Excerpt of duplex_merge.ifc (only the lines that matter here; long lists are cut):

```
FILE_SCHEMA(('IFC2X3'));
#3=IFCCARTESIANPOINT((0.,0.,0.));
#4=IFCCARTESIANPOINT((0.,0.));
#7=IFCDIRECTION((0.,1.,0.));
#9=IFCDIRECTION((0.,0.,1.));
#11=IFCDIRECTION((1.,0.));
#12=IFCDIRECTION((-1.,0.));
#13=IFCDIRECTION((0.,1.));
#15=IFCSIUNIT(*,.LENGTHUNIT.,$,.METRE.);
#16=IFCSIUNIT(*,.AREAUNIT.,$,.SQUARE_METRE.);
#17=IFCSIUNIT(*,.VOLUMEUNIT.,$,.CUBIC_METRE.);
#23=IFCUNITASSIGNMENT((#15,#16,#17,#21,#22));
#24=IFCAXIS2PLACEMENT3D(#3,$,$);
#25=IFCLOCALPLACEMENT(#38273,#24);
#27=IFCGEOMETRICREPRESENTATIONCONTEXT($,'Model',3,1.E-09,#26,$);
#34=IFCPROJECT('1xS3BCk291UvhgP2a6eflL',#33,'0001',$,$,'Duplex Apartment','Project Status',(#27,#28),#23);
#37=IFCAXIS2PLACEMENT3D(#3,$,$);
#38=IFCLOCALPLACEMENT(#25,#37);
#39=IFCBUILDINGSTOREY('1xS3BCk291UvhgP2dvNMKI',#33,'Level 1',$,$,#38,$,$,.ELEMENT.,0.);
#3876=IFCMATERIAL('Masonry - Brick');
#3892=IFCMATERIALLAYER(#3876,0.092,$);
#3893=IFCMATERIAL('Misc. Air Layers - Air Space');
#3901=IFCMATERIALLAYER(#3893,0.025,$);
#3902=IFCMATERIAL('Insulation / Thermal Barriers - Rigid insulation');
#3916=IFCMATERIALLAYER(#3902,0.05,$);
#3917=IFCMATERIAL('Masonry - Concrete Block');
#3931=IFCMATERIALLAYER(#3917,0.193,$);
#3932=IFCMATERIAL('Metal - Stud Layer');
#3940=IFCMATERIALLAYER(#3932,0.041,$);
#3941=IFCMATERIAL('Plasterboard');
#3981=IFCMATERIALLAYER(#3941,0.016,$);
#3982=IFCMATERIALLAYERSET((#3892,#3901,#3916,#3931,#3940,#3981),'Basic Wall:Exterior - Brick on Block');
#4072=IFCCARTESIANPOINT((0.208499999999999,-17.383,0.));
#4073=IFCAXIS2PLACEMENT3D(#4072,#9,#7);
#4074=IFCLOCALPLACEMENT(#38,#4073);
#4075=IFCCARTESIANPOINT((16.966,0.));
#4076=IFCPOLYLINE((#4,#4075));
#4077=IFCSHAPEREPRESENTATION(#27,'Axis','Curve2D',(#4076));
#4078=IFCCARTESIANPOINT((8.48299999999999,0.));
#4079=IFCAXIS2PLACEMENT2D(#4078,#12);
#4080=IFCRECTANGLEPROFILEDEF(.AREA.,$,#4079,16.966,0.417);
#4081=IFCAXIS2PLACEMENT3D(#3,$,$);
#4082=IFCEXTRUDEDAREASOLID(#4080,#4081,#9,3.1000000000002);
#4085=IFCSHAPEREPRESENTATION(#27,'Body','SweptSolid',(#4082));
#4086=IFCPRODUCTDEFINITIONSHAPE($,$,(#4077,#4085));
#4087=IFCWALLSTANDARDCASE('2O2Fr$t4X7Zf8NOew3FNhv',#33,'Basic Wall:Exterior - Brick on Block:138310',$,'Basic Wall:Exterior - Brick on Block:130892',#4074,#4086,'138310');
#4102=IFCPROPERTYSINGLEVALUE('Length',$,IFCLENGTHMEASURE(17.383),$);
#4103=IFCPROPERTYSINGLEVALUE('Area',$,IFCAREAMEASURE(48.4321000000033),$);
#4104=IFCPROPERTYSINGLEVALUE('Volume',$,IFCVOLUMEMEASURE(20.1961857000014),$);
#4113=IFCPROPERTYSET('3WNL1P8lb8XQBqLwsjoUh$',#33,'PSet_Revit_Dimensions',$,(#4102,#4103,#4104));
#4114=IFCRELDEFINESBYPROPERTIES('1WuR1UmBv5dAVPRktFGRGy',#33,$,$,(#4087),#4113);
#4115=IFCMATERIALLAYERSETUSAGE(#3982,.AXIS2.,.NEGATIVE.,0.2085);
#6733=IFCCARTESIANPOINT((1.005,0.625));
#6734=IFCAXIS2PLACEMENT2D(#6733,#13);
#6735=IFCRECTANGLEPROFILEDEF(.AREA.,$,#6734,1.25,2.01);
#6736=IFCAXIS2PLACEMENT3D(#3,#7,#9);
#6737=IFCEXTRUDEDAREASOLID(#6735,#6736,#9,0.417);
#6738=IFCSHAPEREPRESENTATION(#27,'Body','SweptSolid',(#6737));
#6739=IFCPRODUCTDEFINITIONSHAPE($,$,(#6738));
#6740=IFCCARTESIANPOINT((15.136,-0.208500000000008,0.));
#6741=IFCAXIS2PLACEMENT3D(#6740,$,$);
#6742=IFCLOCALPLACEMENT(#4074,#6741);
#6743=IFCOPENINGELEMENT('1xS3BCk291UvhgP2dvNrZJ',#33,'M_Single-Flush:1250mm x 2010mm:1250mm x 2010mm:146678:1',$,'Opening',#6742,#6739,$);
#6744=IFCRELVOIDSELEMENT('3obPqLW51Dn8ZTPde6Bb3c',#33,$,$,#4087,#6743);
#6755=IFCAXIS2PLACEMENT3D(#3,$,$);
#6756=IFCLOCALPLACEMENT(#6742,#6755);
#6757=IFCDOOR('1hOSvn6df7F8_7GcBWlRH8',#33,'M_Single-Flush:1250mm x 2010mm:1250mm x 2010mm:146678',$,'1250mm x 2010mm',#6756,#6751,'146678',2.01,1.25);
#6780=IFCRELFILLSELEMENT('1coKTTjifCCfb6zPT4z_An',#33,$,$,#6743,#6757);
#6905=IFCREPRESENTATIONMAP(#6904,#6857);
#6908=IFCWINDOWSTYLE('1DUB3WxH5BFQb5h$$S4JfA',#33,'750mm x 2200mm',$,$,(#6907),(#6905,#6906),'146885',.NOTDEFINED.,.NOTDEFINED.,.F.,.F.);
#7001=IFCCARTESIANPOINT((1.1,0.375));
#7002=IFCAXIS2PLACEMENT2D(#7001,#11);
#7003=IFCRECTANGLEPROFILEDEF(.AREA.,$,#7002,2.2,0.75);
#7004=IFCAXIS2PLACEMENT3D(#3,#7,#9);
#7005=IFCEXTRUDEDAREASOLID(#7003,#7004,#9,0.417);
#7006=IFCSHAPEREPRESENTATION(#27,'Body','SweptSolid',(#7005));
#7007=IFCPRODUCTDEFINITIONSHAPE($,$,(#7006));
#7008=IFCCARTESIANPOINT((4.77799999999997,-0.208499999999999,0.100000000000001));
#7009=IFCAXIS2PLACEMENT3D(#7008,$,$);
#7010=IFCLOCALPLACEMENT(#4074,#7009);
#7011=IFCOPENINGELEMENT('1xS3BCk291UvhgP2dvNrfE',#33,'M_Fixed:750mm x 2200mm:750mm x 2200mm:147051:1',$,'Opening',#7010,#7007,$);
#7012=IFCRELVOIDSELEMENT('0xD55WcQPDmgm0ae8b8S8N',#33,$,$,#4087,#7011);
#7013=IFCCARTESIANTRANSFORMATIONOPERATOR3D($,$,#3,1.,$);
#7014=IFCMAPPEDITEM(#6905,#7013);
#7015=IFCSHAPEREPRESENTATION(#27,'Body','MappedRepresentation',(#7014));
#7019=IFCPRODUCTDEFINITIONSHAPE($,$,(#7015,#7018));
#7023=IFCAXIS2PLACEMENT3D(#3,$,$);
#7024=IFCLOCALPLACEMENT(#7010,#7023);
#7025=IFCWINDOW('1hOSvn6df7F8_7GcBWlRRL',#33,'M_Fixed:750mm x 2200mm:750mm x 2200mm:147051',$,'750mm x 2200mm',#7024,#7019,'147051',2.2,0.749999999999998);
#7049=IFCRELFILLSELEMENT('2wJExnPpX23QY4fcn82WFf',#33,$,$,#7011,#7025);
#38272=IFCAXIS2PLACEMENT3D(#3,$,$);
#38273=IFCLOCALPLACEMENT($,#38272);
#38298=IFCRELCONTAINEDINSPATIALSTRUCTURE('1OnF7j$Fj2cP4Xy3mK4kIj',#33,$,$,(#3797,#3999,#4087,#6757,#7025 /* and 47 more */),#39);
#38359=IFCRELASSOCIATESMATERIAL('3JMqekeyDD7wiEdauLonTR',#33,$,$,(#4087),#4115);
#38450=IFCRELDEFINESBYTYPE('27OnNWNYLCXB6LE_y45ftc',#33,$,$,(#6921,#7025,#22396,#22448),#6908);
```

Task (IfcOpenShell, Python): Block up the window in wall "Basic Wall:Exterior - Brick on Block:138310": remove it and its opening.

```python
import ifcopenshell
import ifcopenshell.api.feature
import ifcopenshell.api.pset
import ifcopenshell.api.root
import ifcopenshell.geom
import ifcopenshell.util.element
import ifcopenshell.util.shape
import ifcopenshell.util.unit

model = ifcopenshell.open("duplex_merge.ifc")
area_scale = ifcopenshell.util.unit.calculate_unit_scale(model, "AREAUNIT")
volume_scale = ifcopenshell.util.unit.calculate_unit_scale(model, "VOLUMEUNIT")
settings = ifcopenshell.geom.settings()


def volume(element):
    """Net volume in cubic metres, openings subtracted."""
    shape = ifcopenshell.geom.create_shape(settings, element)
    return ifcopenshell.util.shape.get_volume(shape.geometry)


window = model.by_id(7025)
opening = window.FillsVoids[0].RelatingOpeningElement
wall = opening.VoidsElements[0].RelatingBuildingElement
before = volume(wall)

ifcopenshell.api.root.remove_product(model, product=window)
ifcopenshell.api.feature.remove_feature(model, feature=opening)

after = volume(wall)
thickness = 0.417  # wall thickness in metres

# Update the wall's stored quantities.
pset = model.by_id(ifcopenshell.util.element.get_pset(wall, "PSet_Revit_Dimensions", should_inherit=False)["id"])
ifcopenshell.api.pset.edit_pset(model, pset=pset, properties={
    "Area": model.create_entity("IfcAreaMeasure", after / thickness / area_scale),
    "Volume": model.create_entity("IfcVolumeMeasure", after / volume_scale),
})

print(f"wall volume {before:.3f} -> {after:.3f} m3")

model.write("duplex_merge_edited.ifc")
```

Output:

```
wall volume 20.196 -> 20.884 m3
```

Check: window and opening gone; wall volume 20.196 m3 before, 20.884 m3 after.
